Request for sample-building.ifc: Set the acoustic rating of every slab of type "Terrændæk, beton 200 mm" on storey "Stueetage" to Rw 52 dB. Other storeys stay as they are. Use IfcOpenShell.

First a look at what the model holds.

```python
import ifcopenshell
import ifcopenshell.util.element

model = ifcopenshell.open("sample-building.ifc")
print(model.schema)
storey = next(s for s in model.by_type("IfcBuildingStorey") if s.Name == "Stueetage")
slabs = [e for e in ifcopenshell.util.element.get_decomposition(storey) if e.is_a("IfcSlab")]
seen = {}
for e in slabs:
    element_type = ifcopenshell.util.element.get_type(e)
    key = (element_type.Name if element_type != e and element_type else None, ifcopenshell.util.element.get_pset(e, "Pset_SlabCommon", "AcousticRating"))
    seen[key] = seen.get(key, 0) + 1
for (name, value), count in sorted(seen.items(), key=str):
    print(count, "x", name, "|", value)
```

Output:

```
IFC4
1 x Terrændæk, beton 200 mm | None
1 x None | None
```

```python
import ifcopenshell
import ifcopenshell.api.pset
import ifcopenshell.util.element

model = ifcopenshell.open("sample-building.ifc")

storey = next(s for s in model.by_type("IfcBuildingStorey") if s.Name == "Stueetage")
slabs = [e for e in ifcopenshell.util.element.get_decomposition(storey) if e.is_a("IfcSlab")]

count = 0
for e in slabs:
    element_type = ifcopenshell.util.element.get_type(e)
    if element_type in (None, e) or element_type.Name != "Terrændæk, beton 200 mm":
        continue
    # add_pset returns the element's existing set when there is one.
    pset = ifcopenshell.api.pset.add_pset(model, product=e, name="Pset_SlabCommon")
    ifcopenshell.api.pset.edit_pset(model, pset=pset, properties={"AcousticRating": "Rw 52 dB"})
    count += 1

print(count, "slabs updated")

model.write("sample-building-out.ifc")
```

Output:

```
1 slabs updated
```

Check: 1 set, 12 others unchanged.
